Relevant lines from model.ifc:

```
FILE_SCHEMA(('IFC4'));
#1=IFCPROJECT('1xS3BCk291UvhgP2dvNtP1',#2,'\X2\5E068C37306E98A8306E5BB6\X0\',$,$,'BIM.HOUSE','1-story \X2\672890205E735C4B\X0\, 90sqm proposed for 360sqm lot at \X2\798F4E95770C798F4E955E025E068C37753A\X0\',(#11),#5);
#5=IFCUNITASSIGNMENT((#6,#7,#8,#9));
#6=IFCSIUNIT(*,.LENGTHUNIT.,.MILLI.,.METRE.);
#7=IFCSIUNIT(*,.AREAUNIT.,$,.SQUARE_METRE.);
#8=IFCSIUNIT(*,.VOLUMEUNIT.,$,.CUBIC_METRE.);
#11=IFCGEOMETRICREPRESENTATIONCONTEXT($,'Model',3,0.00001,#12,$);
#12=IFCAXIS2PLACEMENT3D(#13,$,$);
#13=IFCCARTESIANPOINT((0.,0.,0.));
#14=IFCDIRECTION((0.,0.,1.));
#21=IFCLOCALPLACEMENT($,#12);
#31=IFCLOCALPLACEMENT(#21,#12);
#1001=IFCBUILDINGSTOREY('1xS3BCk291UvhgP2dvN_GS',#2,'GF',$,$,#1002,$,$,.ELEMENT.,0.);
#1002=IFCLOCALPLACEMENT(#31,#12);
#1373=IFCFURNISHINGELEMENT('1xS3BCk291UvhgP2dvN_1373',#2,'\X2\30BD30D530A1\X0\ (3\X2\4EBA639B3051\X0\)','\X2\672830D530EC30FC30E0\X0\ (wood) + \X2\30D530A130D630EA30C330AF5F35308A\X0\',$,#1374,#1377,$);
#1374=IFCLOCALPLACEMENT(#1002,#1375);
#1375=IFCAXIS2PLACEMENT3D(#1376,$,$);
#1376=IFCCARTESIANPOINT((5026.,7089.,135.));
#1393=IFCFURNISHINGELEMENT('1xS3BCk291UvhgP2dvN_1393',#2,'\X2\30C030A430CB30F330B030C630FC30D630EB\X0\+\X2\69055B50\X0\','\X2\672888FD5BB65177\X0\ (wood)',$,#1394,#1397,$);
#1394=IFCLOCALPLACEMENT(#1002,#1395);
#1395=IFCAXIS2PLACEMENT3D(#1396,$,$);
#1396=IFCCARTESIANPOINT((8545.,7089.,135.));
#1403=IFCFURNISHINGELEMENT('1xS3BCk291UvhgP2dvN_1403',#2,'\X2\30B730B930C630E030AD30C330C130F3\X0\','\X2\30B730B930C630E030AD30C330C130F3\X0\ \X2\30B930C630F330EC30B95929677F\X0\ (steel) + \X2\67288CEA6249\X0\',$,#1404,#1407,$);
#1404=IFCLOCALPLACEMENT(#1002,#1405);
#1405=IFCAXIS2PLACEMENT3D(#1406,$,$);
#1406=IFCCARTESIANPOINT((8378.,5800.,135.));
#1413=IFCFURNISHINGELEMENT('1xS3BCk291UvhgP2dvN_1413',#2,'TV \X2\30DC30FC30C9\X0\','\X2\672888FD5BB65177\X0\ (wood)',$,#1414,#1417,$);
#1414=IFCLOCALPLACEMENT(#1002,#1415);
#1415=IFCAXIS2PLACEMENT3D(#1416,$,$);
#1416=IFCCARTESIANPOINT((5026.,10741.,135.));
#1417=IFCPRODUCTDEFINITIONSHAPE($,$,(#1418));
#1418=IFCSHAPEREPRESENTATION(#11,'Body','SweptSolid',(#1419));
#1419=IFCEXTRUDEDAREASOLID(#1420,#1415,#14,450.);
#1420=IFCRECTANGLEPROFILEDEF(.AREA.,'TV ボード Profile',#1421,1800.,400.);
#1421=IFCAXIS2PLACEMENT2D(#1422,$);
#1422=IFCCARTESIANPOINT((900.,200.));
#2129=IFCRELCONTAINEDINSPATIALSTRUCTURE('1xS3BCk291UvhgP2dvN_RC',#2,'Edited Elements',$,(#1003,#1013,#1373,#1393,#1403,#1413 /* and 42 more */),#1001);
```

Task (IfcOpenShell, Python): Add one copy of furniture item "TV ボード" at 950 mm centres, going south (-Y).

```python
import numpy as np
import ifcopenshell
import ifcopenshell.api.geometry
import ifcopenshell.api.root
import ifcopenshell.util.element
import ifcopenshell.util.placement

model = ifcopenshell.open("model.ifc")


def reuse_history(source, copy):
    """copy_class also copies each property set's owner history, people and application; keep the originals."""
    for rel in copy.IsDefinedBy:
        if rel.is_a("IfcRelDefinesByProperties") and (history := rel.RelatingPropertyDefinition.OwnerHistory):
            rel.RelatingPropertyDefinition.OwnerHistory = source.OwnerHistory
            ifcopenshell.util.element.remove_deep2(model, history)


source = model.by_guid("1xS3BCk291UvhgP2dvN_1413")
base = ifcopenshell.util.placement.get_local_placement(source.ObjectPlacement)
step = np.array([0.0, -1.0, 0.0]) * 950.0

for i in range(1, 2):
    copy = ifcopenshell.api.root.copy_class(model, product=source)
    copy.Representation = ifcopenshell.util.element.copy_deep(
        model, source.Representation, exclude=["IfcGeometricRepresentationContext", "IfcRepresentationMap"]
    )
    reuse_history(source, copy)
    matrix = base.copy()
    matrix[:3, 3] += i * step
    print("added at", matrix[:3, 3].round(3) + 0.0)
    ifcopenshell.api.geometry.edit_object_placement(model, product=copy, matrix=matrix, is_si=False)

model.write("model_rev.ifc")
```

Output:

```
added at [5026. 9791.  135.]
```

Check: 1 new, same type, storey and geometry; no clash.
